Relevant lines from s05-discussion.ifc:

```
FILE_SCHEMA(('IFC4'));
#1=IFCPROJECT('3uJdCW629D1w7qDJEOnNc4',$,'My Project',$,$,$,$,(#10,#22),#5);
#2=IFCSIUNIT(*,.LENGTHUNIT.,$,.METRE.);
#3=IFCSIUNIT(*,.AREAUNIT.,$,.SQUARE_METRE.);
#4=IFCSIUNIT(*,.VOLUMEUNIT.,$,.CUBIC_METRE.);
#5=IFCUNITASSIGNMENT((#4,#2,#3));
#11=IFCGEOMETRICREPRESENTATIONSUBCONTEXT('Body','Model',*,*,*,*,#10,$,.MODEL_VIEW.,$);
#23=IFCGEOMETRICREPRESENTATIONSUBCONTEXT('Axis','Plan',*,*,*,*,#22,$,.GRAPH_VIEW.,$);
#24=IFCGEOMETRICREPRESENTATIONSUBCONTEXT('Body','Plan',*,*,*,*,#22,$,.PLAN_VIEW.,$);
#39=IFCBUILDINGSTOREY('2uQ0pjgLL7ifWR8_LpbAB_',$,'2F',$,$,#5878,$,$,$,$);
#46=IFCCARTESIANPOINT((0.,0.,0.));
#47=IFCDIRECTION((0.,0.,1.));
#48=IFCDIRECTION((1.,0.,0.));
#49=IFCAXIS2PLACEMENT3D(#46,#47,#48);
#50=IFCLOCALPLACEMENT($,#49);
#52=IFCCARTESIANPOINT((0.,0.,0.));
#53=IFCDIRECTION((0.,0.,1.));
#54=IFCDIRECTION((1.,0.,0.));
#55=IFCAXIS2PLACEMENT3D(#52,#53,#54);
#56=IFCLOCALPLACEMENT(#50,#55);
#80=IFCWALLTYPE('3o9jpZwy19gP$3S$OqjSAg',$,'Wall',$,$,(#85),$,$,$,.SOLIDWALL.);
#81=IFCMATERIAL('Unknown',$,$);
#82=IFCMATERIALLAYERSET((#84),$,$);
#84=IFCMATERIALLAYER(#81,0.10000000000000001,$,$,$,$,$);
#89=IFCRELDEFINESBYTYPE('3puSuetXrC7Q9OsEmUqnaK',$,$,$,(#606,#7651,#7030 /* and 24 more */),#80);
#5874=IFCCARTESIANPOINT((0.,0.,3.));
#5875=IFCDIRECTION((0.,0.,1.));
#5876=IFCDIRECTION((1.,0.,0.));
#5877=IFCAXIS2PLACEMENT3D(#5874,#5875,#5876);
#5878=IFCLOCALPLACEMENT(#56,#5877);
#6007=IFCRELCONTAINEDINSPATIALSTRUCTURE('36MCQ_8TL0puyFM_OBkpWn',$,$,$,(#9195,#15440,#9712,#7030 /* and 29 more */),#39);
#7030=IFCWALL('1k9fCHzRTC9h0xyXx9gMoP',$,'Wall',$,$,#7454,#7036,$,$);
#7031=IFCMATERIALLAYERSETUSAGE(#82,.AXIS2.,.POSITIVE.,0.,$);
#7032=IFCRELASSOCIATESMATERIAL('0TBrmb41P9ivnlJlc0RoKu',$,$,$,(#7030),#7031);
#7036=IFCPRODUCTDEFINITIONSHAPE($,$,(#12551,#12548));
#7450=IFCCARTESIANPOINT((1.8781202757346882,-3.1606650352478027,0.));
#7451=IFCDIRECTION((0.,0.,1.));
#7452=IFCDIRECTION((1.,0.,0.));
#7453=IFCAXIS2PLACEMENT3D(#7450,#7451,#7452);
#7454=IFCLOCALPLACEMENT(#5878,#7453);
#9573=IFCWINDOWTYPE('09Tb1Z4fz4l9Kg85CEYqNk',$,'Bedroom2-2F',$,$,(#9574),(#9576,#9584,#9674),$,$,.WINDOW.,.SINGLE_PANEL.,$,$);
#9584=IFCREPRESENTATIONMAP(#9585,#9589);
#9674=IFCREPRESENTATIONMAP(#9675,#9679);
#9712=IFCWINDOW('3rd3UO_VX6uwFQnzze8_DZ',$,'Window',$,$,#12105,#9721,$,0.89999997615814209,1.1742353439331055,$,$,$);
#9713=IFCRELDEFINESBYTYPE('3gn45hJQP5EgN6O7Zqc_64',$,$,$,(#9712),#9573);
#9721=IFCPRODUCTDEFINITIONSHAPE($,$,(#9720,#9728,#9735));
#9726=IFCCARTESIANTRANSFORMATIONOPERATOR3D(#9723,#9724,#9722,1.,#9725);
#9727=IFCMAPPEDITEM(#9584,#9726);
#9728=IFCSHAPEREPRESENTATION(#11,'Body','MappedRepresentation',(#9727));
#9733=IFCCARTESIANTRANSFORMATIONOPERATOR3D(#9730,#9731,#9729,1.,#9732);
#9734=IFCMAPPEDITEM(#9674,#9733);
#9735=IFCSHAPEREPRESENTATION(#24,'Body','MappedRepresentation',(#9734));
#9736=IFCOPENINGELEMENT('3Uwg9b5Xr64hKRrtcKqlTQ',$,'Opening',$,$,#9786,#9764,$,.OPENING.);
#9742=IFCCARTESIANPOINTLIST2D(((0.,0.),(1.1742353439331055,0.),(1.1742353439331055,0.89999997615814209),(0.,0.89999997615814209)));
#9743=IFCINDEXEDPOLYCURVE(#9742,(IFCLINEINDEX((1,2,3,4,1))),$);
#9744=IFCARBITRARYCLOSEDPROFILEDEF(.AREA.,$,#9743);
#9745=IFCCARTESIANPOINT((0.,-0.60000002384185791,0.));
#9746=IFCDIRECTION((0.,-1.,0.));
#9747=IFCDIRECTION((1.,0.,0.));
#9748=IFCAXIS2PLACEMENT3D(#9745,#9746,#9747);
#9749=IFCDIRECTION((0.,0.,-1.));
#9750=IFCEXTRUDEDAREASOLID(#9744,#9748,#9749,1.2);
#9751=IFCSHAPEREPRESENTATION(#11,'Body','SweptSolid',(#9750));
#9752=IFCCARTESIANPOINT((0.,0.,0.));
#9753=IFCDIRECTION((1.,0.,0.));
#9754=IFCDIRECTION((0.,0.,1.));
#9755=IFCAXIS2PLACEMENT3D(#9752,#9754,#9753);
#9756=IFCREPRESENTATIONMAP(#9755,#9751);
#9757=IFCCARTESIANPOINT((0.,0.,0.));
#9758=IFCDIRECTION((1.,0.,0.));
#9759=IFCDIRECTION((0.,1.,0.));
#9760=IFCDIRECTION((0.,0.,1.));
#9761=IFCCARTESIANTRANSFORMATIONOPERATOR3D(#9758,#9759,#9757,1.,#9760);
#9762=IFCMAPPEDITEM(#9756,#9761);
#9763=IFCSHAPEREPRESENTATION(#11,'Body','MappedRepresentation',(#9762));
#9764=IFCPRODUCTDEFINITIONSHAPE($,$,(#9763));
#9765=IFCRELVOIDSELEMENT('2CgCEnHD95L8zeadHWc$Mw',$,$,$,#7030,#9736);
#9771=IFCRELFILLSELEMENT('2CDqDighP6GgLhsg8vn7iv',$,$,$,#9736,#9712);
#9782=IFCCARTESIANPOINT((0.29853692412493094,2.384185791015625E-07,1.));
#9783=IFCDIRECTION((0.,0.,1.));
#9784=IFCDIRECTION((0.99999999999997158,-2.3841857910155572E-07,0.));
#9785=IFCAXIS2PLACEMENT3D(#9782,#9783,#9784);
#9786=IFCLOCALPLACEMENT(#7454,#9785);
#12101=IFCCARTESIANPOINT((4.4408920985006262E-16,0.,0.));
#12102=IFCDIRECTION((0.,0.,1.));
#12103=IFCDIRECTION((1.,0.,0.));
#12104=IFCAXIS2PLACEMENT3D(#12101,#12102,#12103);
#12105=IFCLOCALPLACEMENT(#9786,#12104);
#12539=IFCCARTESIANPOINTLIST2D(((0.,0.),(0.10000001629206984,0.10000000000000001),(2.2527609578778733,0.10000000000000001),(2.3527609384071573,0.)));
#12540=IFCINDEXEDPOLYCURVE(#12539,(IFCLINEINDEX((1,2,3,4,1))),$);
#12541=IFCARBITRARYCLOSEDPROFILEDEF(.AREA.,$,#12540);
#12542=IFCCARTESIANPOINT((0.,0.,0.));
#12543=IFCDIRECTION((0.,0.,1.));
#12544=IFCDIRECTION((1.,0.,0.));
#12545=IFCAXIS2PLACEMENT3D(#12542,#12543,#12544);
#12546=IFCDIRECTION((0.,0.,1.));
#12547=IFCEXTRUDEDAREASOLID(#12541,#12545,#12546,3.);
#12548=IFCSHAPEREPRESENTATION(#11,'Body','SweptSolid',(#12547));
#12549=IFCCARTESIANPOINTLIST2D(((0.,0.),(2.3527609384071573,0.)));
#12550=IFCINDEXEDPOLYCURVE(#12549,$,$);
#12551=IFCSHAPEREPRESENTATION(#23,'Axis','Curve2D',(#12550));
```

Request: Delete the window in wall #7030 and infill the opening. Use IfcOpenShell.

```python
import ifcopenshell
import ifcopenshell.api.feature
import ifcopenshell.api.root
import ifcopenshell.geom
import ifcopenshell.util.shape

model = ifcopenshell.open("s05-discussion.ifc")
settings = ifcopenshell.geom.settings()


def volume(element):
    """Net volume in cubic metres, openings subtracted."""
    shape = ifcopenshell.geom.create_shape(settings, element)
    return ifcopenshell.util.shape.get_volume(shape.geometry)


window = model.by_id(9712)
opening = window.FillsVoids[0].RelatingOpeningElement
wall = opening.VoidsElements[0].RelatingBuildingElement
before = volume(wall)

ifcopenshell.api.root.remove_product(model, product=window)
ifcopenshell.api.feature.remove_feature(model, feature=opening)

after = volume(wall)

print(f"wall volume {before:.3f} -> {after:.3f} m3")

model.write("s05-discussion-out.ifc")
```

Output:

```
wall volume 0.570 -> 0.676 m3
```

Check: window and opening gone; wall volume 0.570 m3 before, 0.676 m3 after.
